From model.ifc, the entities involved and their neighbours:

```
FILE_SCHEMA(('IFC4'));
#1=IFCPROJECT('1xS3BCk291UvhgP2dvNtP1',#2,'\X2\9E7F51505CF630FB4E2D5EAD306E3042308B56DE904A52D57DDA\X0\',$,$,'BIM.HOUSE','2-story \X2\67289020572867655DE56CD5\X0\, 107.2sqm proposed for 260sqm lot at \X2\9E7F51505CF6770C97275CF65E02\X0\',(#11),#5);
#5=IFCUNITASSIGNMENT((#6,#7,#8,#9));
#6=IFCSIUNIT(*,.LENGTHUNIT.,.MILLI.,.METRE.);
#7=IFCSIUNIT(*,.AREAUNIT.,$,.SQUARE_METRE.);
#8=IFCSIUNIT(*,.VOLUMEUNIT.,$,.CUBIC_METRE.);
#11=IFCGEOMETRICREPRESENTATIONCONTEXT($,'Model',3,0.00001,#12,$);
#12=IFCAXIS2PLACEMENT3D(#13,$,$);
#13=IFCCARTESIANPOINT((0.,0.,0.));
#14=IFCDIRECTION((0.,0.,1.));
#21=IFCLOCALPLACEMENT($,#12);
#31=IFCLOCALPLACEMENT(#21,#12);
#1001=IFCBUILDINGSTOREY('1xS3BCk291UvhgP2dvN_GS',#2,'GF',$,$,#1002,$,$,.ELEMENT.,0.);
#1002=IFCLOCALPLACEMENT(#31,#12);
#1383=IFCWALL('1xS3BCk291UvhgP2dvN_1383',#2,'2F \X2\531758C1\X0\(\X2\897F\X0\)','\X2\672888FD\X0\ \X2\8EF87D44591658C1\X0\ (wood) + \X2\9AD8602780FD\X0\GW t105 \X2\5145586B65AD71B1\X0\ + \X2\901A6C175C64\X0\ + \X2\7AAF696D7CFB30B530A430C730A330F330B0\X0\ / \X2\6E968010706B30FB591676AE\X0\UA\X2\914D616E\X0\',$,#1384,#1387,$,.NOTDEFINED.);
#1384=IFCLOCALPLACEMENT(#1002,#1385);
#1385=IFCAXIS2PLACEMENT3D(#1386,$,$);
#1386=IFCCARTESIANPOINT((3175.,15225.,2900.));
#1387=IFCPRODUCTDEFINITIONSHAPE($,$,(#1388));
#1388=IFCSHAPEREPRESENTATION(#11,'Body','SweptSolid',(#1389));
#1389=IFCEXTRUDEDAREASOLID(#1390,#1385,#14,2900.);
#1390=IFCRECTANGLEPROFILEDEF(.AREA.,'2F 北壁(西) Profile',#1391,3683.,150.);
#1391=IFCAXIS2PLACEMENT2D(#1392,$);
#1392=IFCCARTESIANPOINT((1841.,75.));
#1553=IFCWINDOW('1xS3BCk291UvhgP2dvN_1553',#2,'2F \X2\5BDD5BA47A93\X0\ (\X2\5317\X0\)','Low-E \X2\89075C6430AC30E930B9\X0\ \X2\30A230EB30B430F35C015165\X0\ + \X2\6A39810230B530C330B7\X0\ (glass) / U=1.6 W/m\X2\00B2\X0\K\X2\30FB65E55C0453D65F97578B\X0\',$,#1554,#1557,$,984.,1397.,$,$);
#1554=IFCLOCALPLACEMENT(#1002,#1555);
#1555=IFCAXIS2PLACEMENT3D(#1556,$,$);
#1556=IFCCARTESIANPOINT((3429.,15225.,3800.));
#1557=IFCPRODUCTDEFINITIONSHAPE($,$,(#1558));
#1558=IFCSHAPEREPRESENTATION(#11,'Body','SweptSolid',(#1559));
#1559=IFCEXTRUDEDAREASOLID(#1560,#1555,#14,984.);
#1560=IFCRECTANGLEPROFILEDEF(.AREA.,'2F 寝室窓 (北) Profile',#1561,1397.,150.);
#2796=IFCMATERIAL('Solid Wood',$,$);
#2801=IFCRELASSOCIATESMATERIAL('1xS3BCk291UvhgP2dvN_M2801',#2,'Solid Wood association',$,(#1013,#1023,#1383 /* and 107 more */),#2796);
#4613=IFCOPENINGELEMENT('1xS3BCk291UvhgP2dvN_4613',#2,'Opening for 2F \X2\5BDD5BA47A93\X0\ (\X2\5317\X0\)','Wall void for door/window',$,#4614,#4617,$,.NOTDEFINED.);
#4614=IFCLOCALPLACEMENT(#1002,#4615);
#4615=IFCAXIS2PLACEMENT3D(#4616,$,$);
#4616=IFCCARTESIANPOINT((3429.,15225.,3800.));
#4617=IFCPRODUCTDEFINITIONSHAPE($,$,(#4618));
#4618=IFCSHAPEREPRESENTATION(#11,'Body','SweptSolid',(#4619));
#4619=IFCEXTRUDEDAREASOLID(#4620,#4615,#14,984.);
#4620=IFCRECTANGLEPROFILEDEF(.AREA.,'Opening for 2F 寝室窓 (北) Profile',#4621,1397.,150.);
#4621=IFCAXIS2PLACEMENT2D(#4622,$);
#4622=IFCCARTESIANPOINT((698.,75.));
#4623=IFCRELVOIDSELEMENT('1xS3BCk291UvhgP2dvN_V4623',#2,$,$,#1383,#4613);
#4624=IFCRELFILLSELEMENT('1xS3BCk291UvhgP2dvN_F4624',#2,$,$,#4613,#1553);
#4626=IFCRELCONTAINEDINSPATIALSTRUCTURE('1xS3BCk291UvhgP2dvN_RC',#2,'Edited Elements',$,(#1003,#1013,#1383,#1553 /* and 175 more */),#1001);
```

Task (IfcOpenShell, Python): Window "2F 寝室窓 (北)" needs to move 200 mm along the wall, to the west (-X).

```python
import ifcopenshell
import ifcopenshell.api.geometry
import ifcopenshell.util.placement
import ifcopenshell.util.unit

model = ifcopenshell.open("model.ifc")
unit_scale = ifcopenshell.util.unit.calculate_unit_scale(model)

window = model.by_id(1553)
opening = window.FillsVoids[0].RelatingOpeningElement
wall = opening.VoidsElements[0].RelatingBuildingElement

wall_matrix = ifcopenshell.util.placement.get_local_placement(wall.ObjectPlacement)
shift = wall_matrix[:3, 0] * -0.2 / unit_scale
before = ifcopenshell.util.placement.get_local_placement(window.ObjectPlacement)[:3, 3].copy()

# The window is not placed relative to its opening, so move both.
for product in (opening, window):
    matrix = ifcopenshell.util.placement.get_local_placement(product.ObjectPlacement)
    matrix[:3, 3] += shift
    ifcopenshell.api.geometry.edit_object_placement(model, product=product, matrix=matrix, is_si=False)

after = ifcopenshell.util.placement.get_local_placement(window.ObjectPlacement)[:3, 3]
print("window moved by", (after - before).round(3) + 0.0)

model.write("model_rev.ifc")
```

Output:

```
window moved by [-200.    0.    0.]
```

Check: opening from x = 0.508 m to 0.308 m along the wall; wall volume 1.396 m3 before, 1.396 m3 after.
